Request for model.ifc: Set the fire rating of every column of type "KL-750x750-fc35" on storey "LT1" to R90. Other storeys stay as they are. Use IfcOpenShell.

First a look at what the model holds.

```python
import ifcopenshell
import ifcopenshell.util.element

model = ifcopenshell.open("model.ifc")
print(model.schema)
storey = next(s for s in model.by_type("IfcBuildingStorey") if s.Name == "LT1")
columns = [e for e in ifcopenshell.util.element.get_decomposition(storey) if e.is_a("IfcColumn")]
seen = {}
for e in columns:
    element_type = ifcopenshell.util.element.get_type(e)
    key = (element_type.Name if element_type != e and element_type else None, ifcopenshell.util.element.get_pset(e, "Pset_ColumnCommon", "FireRating"))
    seen[key] = seen.get(key, 0) + 1
for (name, value), count in sorted(seen.items(), key=str):
    print(count, "x", name, "|", value)
```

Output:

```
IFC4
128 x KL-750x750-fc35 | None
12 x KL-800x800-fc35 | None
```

```python
import ifcopenshell
import ifcopenshell.api.pset
import ifcopenshell.util.element

model = ifcopenshell.open("model.ifc")

storey = next(s for s in model.by_type("IfcBuildingStorey") if s.Name == "LT1")
columns = [e for e in ifcopenshell.util.element.get_decomposition(storey) if e.is_a("IfcColumn")]

count = 0
for e in columns:
    element_type = ifcopenshell.util.element.get_type(e)
    if element_type in (None, e) or element_type.Name != "KL-750x750-fc35":
        continue
    # add_pset returns the element's existing set when there is one.
    pset = ifcopenshell.api.pset.add_pset(model, product=e, name="Pset_ColumnCommon")
    ifcopenshell.api.pset.edit_pset(model, pset=pset, properties={"FireRating": "R90"})
    count += 1

print(count, "columns updated")

model.write("model_updated.ifc")
```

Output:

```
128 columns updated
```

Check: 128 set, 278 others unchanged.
